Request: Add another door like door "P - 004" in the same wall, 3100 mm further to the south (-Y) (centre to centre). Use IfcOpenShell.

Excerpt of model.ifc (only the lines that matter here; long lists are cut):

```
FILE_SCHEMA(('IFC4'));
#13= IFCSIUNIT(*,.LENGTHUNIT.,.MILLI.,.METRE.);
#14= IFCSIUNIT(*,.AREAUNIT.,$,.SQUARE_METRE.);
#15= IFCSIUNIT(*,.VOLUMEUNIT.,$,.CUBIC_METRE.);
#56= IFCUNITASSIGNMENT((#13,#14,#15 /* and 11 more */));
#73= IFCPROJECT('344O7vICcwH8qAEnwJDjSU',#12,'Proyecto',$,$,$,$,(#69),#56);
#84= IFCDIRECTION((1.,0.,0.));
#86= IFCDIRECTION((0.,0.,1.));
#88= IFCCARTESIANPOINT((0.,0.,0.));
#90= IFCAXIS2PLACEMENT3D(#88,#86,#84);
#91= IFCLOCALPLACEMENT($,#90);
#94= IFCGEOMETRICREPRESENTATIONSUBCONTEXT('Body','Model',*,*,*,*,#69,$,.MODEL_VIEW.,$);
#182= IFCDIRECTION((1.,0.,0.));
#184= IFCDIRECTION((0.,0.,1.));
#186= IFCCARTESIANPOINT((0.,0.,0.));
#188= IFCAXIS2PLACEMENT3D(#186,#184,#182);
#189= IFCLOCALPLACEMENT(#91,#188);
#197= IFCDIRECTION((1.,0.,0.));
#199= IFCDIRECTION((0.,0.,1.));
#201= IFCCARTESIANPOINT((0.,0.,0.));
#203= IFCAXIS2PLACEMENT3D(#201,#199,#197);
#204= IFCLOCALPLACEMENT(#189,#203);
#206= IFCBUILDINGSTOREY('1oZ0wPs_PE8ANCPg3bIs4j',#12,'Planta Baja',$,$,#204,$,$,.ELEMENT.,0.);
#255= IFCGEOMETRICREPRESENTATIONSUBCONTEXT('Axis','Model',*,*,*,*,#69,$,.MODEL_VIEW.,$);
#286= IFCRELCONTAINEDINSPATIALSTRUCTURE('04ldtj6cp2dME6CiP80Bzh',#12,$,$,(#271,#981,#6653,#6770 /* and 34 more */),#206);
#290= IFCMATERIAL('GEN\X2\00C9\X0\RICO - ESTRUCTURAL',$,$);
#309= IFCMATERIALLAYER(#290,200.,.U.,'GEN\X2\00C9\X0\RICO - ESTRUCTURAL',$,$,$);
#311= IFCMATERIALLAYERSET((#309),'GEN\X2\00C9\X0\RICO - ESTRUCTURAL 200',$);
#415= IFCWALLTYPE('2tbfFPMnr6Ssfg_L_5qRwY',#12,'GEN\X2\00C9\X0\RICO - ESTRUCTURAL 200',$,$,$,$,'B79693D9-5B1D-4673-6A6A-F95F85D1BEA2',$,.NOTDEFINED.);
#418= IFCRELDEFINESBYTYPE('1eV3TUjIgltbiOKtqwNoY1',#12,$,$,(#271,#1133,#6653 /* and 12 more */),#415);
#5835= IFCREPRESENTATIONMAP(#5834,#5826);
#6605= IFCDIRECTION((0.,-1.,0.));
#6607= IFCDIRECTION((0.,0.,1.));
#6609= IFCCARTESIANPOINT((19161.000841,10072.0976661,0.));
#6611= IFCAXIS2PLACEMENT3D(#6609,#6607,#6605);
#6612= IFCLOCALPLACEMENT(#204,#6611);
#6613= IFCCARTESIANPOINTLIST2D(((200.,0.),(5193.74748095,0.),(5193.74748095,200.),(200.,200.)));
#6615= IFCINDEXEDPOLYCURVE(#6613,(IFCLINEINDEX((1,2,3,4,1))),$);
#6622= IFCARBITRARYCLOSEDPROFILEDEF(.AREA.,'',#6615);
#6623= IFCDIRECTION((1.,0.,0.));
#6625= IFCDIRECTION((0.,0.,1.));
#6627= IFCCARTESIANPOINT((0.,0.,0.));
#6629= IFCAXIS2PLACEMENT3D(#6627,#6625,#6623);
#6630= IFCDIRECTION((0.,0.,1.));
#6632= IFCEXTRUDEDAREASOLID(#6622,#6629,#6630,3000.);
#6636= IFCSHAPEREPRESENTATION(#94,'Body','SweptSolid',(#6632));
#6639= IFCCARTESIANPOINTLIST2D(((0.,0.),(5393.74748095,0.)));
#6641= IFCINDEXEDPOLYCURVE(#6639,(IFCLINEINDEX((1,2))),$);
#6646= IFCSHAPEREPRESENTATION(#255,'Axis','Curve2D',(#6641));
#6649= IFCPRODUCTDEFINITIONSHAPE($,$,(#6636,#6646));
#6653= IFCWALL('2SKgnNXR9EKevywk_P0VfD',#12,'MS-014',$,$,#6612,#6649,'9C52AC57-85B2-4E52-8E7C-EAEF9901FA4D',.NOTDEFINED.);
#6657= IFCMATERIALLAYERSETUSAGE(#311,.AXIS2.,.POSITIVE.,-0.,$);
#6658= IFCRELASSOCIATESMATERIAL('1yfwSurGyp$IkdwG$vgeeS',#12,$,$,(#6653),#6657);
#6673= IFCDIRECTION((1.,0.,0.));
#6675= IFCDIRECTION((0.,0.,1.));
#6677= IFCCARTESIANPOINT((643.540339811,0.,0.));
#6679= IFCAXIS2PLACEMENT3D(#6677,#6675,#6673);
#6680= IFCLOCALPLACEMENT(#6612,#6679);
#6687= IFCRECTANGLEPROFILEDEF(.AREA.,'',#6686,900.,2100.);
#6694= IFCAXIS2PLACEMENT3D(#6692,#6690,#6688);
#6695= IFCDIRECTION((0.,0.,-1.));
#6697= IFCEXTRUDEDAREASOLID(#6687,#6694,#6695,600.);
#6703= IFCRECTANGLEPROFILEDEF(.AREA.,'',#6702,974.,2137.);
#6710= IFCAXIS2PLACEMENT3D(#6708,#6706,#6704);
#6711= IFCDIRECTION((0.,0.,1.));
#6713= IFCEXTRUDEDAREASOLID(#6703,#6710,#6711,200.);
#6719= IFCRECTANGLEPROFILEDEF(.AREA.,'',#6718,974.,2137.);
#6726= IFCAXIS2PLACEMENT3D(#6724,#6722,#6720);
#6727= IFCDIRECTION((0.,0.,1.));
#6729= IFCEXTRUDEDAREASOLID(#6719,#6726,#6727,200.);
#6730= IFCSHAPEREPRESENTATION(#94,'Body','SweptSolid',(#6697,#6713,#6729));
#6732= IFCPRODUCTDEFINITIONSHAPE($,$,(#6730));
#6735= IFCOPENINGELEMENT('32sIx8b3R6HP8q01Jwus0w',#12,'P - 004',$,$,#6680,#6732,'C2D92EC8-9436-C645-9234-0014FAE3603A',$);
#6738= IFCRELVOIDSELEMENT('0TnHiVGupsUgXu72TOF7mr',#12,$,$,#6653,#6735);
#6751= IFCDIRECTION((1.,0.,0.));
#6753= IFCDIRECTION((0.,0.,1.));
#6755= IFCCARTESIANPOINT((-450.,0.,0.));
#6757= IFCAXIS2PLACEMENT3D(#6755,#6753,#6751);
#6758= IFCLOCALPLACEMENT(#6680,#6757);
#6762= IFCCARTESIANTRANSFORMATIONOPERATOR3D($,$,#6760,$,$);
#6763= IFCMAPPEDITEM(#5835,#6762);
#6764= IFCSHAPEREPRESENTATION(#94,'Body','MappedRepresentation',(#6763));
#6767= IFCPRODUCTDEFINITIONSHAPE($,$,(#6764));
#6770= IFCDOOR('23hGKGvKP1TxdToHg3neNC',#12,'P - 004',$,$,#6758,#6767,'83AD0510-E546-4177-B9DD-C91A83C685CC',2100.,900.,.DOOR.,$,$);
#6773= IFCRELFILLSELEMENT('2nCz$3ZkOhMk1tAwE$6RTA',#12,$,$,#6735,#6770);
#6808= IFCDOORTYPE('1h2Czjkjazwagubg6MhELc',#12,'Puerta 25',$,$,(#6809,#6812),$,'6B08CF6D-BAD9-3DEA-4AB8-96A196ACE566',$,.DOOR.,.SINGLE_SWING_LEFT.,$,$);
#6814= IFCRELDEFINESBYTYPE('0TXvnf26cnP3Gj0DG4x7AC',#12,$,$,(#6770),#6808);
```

```python
import ifcopenshell
import ifcopenshell.api.feature
import ifcopenshell.api.geometry
import ifcopenshell.api.root
import ifcopenshell.geom
import ifcopenshell.util.element
import ifcopenshell.util.placement
import ifcopenshell.util.shape
import ifcopenshell.util.unit

model = ifcopenshell.open("model.ifc")
unit_scale = ifcopenshell.util.unit.calculate_unit_scale(model)
settings = ifcopenshell.geom.settings()


def volume(element):
    """Net volume in cubic metres, openings subtracted."""
    shape = ifcopenshell.geom.create_shape(settings, element)
    return ifcopenshell.util.shape.get_volume(shape.geometry)


def reuse_history(source, copy):
    """copy_class also copies each property set's owner history, people and application; keep the originals."""
    for rel in copy.IsDefinedBy:
        if rel.is_a("IfcRelDefinesByProperties") and (history := rel.RelatingPropertyDefinition.OwnerHistory):
            rel.RelatingPropertyDefinition.OwnerHistory = source.OwnerHistory
            ifcopenshell.util.element.remove_deep2(model, history)


door = model.by_guid("23hGKGvKP1TxdToHg3neNC")
opening = door.FillsVoids[0].RelatingOpeningElement
wall = opening.VoidsElements[0].RelatingBuildingElement
before = volume(wall)
shift = ifcopenshell.util.placement.get_local_placement(wall.ObjectPlacement)[:3, 0] * 3.1 / unit_scale

# copy_class copies the void relationship, type, container and properties, but no geometry.
new_opening = ifcopenshell.api.root.copy_class(model, product=opening)
new_opening.Representation = ifcopenshell.util.element.copy_deep(
    model, opening.Representation, exclude=["IfcGeometricRepresentationContext", "IfcRepresentationMap"]
)
new_opening.Tag = None
new_door = ifcopenshell.api.root.copy_class(model, product=door)
new_door.Representation = ifcopenshell.util.element.copy_deep(
    model, door.Representation, exclude=["IfcGeometricRepresentationContext", "IfcRepresentationMap"]
)
new_door.Tag = None
reuse_history(door, new_door)
ifcopenshell.api.feature.add_filling(model, opening=new_opening, element=new_door)

for old, new in ((opening, new_opening), (door, new_door)):
    matrix = ifcopenshell.util.placement.get_local_placement(old.ObjectPlacement)
    matrix[:3, 3] += shift
    ifcopenshell.api.geometry.edit_object_placement(model, product=new, matrix=matrix, is_si=False)

after = volume(wall)

print(f"wall volume {before:.3f} -> {after:.3f} m3")

model.write("model_updated.ifc")
```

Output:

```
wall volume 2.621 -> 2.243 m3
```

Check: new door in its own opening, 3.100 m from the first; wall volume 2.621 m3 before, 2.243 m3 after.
